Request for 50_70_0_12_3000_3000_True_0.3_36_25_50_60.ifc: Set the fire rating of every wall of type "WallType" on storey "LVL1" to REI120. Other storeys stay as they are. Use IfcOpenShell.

First a look at what the model holds.

```python
import ifcopenshell
import ifcopenshell.util.element

model = ifcopenshell.open("50_70_0_12_3000_3000_True_0.3_36_25_50_60.ifc")
print(model.schema)
storey = next(s for s in model.by_type("IfcBuildingStorey") if s.Name == "LVL1")
walls = [e for e in ifcopenshell.util.element.get_decomposition(storey) if e.is_a("IfcWall")]
seen = {}
for e in walls:
    element_type = ifcopenshell.util.element.get_type(e)
    key = (element_type.Name if element_type != e and element_type else None, ifcopenshell.util.element.get_pset(e, "Pset_WallCommon", "FireRating"))
    seen[key] = seen.get(key, 0) + 1
for (name, value), count in sorted(seen.items(), key=str):
    print(count, "x", name, "|", value)
```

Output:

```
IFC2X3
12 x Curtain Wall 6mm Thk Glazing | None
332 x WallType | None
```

```python
import ifcopenshell
import ifcopenshell.api.pset
import ifcopenshell.util.element

model = ifcopenshell.open("50_70_0_12_3000_3000_True_0.3_36_25_50_60.ifc")

storey = next(s for s in model.by_type("IfcBuildingStorey") if s.Name == "LVL1")
walls = [e for e in ifcopenshell.util.element.get_decomposition(storey) if e.is_a("IfcWall")]

count = 0
for e in walls:
    element_type = ifcopenshell.util.element.get_type(e)
    if element_type in (None, e) or element_type.Name != "WallType":
        continue
    # add_pset returns the element's existing set when there is one.
    pset = ifcopenshell.api.pset.add_pset(model, product=e, name="Pset_WallCommon")
    ifcopenshell.api.pset.edit_pset(model, pset=pset, properties={"FireRating": "REI120"})
    count += 1

print(count, "walls updated")

model.write("50_70_0_12_3000_3000_True_0.3_36_25_50_60_edited.ifc")
```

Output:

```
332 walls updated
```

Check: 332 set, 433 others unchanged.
